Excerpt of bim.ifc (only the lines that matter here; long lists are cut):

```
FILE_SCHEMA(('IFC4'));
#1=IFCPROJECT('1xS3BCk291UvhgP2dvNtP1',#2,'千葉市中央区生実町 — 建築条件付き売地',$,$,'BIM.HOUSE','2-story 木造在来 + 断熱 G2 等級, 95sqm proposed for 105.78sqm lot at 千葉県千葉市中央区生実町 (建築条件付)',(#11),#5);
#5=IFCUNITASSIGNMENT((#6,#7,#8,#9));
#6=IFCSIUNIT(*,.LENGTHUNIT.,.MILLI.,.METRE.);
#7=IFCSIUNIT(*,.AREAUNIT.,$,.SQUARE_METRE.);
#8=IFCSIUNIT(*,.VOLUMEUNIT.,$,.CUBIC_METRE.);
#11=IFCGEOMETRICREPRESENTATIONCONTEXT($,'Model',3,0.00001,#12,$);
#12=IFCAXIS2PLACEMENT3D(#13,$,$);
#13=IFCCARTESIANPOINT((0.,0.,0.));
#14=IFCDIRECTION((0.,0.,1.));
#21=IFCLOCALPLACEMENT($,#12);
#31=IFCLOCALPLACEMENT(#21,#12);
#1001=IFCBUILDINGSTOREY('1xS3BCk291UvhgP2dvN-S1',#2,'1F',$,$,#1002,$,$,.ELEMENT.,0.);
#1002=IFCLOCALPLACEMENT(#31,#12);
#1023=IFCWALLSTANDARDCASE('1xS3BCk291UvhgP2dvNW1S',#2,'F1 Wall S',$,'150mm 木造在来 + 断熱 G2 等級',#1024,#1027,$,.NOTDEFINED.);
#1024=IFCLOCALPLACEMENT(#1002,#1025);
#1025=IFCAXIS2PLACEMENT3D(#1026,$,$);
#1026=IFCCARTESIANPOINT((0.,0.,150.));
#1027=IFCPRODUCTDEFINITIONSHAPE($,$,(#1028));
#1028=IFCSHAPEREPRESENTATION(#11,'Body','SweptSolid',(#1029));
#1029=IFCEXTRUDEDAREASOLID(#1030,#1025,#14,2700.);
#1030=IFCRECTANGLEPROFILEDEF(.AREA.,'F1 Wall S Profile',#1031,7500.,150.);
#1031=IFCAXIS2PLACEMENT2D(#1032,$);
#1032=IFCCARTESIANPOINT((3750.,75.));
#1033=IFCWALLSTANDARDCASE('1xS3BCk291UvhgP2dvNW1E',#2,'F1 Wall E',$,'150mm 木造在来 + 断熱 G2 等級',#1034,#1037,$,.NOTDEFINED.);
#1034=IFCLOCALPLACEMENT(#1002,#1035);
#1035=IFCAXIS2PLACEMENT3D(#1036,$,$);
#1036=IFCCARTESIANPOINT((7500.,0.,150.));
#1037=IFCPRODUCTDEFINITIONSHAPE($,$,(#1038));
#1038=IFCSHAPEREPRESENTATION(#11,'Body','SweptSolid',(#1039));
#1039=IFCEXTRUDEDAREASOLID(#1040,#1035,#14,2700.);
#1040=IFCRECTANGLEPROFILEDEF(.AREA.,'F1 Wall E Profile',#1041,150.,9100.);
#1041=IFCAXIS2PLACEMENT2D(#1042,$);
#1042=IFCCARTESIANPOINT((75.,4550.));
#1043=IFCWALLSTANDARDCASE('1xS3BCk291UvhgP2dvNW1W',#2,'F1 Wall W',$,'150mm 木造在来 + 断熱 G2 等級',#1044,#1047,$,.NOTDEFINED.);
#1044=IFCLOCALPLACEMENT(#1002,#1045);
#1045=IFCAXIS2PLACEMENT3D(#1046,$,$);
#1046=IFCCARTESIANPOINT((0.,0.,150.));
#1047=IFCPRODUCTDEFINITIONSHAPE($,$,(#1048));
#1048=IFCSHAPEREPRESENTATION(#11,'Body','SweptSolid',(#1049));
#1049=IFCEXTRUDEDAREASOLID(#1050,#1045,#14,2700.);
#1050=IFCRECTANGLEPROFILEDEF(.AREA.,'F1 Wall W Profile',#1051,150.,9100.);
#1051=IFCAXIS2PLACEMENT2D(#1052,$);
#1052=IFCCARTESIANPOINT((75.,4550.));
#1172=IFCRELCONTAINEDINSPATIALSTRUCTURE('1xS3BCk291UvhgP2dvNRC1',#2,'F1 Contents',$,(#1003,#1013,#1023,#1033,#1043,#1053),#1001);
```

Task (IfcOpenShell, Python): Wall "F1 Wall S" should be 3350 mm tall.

```python
import ifcopenshell
import ifcopenshell.geom
import ifcopenshell.util.shape

model = ifcopenshell.open("bim.ifc")
settings = ifcopenshell.geom.settings()


def volume(element):
    """Net volume in cubic metres, openings subtracted."""
    shape = ifcopenshell.geom.create_shape(settings, element)
    return ifcopenshell.util.shape.get_volume(shape.geometry)


wall = model.by_guid("1xS3BCk291UvhgP2dvNW1S")
before = volume(wall)

body = next(r for r in wall.Representation.Representations if r.RepresentationIdentifier == "Body")
solid = body.Items[0]
old_height = solid.Depth
solid.Depth = 3350.0
after = volume(wall)

print(f"height {old_height:g} -> {solid.Depth:g}, volume {before:.3f} -> {after:.3f} m3")

model.write("bim_rev.ifc")
```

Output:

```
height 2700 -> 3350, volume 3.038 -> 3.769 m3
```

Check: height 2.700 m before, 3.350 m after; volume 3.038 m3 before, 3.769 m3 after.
